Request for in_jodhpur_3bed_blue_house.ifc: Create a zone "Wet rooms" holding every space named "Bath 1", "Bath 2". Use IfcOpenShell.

First a look at what the model holds.

```python
import ifcopenshell

model = ifcopenshell.open("in_jodhpur_3bed_blue_house.ifc")
print(model.schema)
seen = {}
for space in model.by_type("IfcSpace"):
    seen[space.LongName] = seen.get(space.LongName, 0) + 1
for name, count in sorted(seen.items(), key=str):
    print(count, "x", name)
print("zones:", [z.Name for z in model.by_type("IfcZone")][:20])
```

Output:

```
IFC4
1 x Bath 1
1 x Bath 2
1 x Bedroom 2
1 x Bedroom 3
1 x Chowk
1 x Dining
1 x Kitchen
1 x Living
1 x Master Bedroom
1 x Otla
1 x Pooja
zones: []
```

```python
import ifcopenshell
import ifcopenshell.api.group
import ifcopenshell.api.root

model = ifcopenshell.open("in_jodhpur_3bed_blue_house.ifc")

names = {"Bath 1", "Bath 2"}
spaces = [s for s in model.by_type("IfcSpace") if s.LongName in names]

zone = ifcopenshell.api.root.create_entity(model, ifc_class="IfcZone", name="Wet rooms")
ifcopenshell.api.group.assign_group(model, products=spaces, group=zone)
print(len(spaces), "spaces in", zone.Name)

model.write("in_jodhpur_3bed_blue_house_rev.ifc")
```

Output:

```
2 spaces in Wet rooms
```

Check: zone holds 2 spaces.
